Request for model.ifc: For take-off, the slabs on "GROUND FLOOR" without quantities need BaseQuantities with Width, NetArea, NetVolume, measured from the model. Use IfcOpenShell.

First a look at what the model holds.

```python
import ifcopenshell
import ifcopenshell.util.element
import ifcopenshell.util.unit

model = ifcopenshell.open("model.ifc")
print(model.schema)
for unit_type in ("LENGTHUNIT", "AREAUNIT", "VOLUMEUNIT"):
    print(unit_type, ifcopenshell.util.unit.calculate_unit_scale(model, unit_type))
storey = next(s for s in model.by_type("IfcBuildingStorey") if s.Name == "GROUND FLOOR")
slabs = [e for e in ifcopenshell.util.element.get_decomposition(storey) if e.is_a("IfcSlab")]
for e in sorted(slabs, key=lambda e: e.id()):
    print(e.id(), e.is_a(), e.Name, list(ifcopenshell.util.element.get_psets(e, qtos_only=True)), sep=" | ")
```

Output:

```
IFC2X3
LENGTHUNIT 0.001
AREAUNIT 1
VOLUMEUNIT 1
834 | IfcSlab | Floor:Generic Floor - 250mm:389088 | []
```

```python
import ifcopenshell
import ifcopenshell.api.pset
import ifcopenshell.geom
import ifcopenshell.util.element
import ifcopenshell.util.shape
import ifcopenshell.util.unit

model = ifcopenshell.open("model.ifc")
unit_scale = ifcopenshell.util.unit.calculate_unit_scale(model)
area_scale = ifcopenshell.util.unit.calculate_unit_scale(model, "AREAUNIT")
volume_scale = ifcopenshell.util.unit.calculate_unit_scale(model, "VOLUMEUNIT")
settings = ifcopenshell.geom.settings()

storey = next(s for s in model.by_type("IfcBuildingStorey") if s.Name == "GROUND FLOOR")
slabs = [e for e in ifcopenshell.util.element.get_decomposition(storey) if e.is_a("IfcSlab")]

for e in sorted(slabs, key=lambda e: e.id()):
    if ifcopenshell.util.element.get_psets(e, qtos_only=True, should_inherit=False):
        continue
    # Geometry comes back in metres, in the element's own axes.
    shape = ifcopenshell.geom.create_shape(settings, e)
    values = {
        "Width": ifcopenshell.util.shape.get_z(shape.geometry) / unit_scale,
        "NetArea": ifcopenshell.util.shape.get_footprint_area(shape.geometry) / area_scale,
        "NetVolume": ifcopenshell.util.shape.get_volume(shape.geometry) / volume_scale,
    }
    qto = ifcopenshell.api.pset.add_qto(model, product=e, name="BaseQuantities")
    ifcopenshell.api.pset.edit_qto(model, qto=qto, properties=values)
    print(e.id(), {k: round(v, 3) for k, v in values.items()})

model.write("model_edited.ifc")
```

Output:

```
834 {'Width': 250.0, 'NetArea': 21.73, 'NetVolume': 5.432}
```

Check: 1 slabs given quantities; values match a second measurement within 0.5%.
